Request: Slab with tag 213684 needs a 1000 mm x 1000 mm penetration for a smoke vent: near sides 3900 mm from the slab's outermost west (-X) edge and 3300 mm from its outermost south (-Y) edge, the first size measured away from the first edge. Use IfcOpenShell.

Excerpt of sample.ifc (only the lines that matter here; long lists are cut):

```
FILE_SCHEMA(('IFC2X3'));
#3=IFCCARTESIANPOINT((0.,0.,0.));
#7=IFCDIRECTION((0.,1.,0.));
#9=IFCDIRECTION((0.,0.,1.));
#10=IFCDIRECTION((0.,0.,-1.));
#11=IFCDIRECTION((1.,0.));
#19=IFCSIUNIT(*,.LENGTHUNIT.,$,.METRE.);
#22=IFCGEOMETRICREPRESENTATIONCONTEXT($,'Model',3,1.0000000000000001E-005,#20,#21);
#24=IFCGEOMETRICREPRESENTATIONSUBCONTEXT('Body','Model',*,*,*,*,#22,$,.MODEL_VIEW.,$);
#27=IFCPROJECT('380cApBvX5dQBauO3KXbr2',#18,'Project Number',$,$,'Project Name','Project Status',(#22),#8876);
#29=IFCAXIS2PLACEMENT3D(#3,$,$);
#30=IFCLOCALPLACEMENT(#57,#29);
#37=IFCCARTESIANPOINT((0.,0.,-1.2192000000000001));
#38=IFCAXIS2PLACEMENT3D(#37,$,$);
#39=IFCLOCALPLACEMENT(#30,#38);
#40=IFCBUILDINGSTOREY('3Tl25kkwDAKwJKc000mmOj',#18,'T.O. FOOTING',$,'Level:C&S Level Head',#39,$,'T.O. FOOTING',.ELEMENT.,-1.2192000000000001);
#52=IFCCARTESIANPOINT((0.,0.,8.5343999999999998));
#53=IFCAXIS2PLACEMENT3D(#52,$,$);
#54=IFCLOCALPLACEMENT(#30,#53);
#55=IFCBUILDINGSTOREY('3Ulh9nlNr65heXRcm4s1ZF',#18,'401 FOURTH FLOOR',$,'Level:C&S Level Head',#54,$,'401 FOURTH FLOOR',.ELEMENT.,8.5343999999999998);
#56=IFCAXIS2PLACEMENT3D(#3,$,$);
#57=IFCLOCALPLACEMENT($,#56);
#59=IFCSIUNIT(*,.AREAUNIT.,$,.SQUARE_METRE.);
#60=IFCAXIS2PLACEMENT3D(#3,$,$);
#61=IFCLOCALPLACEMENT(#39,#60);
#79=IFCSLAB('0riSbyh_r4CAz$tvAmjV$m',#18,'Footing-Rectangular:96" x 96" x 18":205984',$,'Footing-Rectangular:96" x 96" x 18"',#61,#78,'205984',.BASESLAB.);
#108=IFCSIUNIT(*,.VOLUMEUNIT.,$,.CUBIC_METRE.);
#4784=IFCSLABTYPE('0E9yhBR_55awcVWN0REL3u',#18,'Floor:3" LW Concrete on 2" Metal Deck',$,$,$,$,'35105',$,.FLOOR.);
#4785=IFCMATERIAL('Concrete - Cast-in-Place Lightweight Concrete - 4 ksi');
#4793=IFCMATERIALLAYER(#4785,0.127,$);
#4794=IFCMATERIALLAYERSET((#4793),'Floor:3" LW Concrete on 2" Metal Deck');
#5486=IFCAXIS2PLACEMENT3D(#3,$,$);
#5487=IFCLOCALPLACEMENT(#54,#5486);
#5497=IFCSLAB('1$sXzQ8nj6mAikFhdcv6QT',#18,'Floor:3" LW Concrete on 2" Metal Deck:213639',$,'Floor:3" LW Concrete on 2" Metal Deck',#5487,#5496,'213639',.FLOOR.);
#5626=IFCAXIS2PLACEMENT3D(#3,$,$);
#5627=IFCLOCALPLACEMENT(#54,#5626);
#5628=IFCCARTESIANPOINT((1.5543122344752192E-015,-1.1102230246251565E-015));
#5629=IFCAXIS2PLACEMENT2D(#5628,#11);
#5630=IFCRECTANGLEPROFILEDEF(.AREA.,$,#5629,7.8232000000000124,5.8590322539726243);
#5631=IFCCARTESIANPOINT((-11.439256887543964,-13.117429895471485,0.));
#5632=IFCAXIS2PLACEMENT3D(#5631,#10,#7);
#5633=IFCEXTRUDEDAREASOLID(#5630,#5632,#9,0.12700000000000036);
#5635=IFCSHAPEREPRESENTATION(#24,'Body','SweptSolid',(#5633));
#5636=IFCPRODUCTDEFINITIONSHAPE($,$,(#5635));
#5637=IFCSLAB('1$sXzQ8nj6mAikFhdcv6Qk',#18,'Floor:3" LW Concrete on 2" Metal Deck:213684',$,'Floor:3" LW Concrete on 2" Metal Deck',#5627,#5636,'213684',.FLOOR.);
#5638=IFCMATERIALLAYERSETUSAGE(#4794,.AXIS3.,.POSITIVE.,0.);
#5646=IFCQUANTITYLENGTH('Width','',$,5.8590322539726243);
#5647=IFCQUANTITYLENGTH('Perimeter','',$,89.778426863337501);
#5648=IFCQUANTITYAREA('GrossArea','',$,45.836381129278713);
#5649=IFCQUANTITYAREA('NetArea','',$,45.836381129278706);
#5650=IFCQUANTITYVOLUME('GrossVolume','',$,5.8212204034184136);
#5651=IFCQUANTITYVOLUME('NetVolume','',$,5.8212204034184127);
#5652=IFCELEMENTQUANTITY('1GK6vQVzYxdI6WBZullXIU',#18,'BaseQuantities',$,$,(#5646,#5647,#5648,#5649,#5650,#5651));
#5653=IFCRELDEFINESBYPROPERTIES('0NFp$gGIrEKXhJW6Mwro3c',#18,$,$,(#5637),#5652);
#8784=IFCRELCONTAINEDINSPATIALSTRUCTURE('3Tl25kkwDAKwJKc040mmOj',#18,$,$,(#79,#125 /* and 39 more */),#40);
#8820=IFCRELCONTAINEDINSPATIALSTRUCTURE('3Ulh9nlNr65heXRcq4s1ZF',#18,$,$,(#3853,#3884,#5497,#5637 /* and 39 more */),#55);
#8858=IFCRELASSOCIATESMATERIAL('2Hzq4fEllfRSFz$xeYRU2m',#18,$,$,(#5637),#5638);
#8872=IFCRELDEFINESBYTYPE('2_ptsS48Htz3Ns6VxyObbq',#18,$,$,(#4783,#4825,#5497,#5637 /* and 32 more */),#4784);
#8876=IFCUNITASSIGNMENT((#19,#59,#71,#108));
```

```python
import numpy as np
import ifcopenshell
import ifcopenshell.api.feature
import ifcopenshell.api.geometry
import ifcopenshell.api.pset
import ifcopenshell.api.root
import ifcopenshell.geom
import ifcopenshell.util.element
import ifcopenshell.util.placement
import ifcopenshell.util.representation
import ifcopenshell.util.shape
import ifcopenshell.util.unit

model = ifcopenshell.open("sample.ifc")
unit_scale = ifcopenshell.util.unit.calculate_unit_scale(model)
area_scale = ifcopenshell.util.unit.calculate_unit_scale(model, "AREAUNIT")
volume_scale = ifcopenshell.util.unit.calculate_unit_scale(model, "VOLUMEUNIT")
settings = ifcopenshell.geom.settings()


def volume(element):
    """Net volume in cubic metres, openings subtracted."""
    shape = ifcopenshell.geom.create_shape(settings, element)
    return ifcopenshell.util.shape.get_volume(shape.geometry)


slab = model.by_guid("1$sXzQ8nj6mAikFhdcv6Qk")
before = volume(slab)

# Extent in the slab's own axes, in metres. The edges named are its -X and -Y sides.
slab_shape = ifcopenshell.geom.create_shape(settings, slab)
vertices = ifcopenshell.util.shape.get_vertices(slab_shape.geometry)
x_min, y_min, bottom = vertices.min(axis=0)
top = vertices[:, 2].max()

opening = ifcopenshell.api.root.create_entity(model, ifc_class="IfcOpeningElement", name="Smoke vent opening")
context = ifcopenshell.util.representation.get_context(model, "Model", "Body", "MODEL_VIEW")
width, depth = 1, 1
outline = [(0.0, 0.0), (width, 0.0), (width, depth), (0.0, depth), (0.0, 0.0)]
# Overshoot both faces by 50 mm so the cut is clean.
shape = ifcopenshell.api.geometry.add_slab_representation(
    model, context=context, depth=top - bottom + 0.1, polyline=outline
)
ifcopenshell.api.geometry.assign_representation(model, product=opening, representation=shape)

matrix = ifcopenshell.util.placement.get_local_placement(slab.ObjectPlacement)
matrix[:, 3] = matrix @ np.append(np.array([x_min + 3.9, y_min + 3.3, bottom - 0.05]) / unit_scale, 1.0)
ifcopenshell.api.geometry.edit_object_placement(model, product=opening, matrix=matrix, is_si=False)
ifcopenshell.api.feature.add_feature(model, feature=opening, element=slab)

after = volume(slab)

# Update the slab's stored quantities.
qto = model.by_id(ifcopenshell.util.element.get_pset(slab, "BaseQuantities", should_inherit=False)["id"])
ifcopenshell.api.pset.edit_qto(model, qto=qto, properties={
    "NetArea": after / (top - bottom) / area_scale,
    "NetVolume": after / volume_scale,
})

print(f"slab volume {before:.3f} -> {after:.3f} m3")

model.write("sample_edited.ifc")
```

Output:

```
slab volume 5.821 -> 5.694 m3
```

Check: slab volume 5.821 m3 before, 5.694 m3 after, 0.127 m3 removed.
